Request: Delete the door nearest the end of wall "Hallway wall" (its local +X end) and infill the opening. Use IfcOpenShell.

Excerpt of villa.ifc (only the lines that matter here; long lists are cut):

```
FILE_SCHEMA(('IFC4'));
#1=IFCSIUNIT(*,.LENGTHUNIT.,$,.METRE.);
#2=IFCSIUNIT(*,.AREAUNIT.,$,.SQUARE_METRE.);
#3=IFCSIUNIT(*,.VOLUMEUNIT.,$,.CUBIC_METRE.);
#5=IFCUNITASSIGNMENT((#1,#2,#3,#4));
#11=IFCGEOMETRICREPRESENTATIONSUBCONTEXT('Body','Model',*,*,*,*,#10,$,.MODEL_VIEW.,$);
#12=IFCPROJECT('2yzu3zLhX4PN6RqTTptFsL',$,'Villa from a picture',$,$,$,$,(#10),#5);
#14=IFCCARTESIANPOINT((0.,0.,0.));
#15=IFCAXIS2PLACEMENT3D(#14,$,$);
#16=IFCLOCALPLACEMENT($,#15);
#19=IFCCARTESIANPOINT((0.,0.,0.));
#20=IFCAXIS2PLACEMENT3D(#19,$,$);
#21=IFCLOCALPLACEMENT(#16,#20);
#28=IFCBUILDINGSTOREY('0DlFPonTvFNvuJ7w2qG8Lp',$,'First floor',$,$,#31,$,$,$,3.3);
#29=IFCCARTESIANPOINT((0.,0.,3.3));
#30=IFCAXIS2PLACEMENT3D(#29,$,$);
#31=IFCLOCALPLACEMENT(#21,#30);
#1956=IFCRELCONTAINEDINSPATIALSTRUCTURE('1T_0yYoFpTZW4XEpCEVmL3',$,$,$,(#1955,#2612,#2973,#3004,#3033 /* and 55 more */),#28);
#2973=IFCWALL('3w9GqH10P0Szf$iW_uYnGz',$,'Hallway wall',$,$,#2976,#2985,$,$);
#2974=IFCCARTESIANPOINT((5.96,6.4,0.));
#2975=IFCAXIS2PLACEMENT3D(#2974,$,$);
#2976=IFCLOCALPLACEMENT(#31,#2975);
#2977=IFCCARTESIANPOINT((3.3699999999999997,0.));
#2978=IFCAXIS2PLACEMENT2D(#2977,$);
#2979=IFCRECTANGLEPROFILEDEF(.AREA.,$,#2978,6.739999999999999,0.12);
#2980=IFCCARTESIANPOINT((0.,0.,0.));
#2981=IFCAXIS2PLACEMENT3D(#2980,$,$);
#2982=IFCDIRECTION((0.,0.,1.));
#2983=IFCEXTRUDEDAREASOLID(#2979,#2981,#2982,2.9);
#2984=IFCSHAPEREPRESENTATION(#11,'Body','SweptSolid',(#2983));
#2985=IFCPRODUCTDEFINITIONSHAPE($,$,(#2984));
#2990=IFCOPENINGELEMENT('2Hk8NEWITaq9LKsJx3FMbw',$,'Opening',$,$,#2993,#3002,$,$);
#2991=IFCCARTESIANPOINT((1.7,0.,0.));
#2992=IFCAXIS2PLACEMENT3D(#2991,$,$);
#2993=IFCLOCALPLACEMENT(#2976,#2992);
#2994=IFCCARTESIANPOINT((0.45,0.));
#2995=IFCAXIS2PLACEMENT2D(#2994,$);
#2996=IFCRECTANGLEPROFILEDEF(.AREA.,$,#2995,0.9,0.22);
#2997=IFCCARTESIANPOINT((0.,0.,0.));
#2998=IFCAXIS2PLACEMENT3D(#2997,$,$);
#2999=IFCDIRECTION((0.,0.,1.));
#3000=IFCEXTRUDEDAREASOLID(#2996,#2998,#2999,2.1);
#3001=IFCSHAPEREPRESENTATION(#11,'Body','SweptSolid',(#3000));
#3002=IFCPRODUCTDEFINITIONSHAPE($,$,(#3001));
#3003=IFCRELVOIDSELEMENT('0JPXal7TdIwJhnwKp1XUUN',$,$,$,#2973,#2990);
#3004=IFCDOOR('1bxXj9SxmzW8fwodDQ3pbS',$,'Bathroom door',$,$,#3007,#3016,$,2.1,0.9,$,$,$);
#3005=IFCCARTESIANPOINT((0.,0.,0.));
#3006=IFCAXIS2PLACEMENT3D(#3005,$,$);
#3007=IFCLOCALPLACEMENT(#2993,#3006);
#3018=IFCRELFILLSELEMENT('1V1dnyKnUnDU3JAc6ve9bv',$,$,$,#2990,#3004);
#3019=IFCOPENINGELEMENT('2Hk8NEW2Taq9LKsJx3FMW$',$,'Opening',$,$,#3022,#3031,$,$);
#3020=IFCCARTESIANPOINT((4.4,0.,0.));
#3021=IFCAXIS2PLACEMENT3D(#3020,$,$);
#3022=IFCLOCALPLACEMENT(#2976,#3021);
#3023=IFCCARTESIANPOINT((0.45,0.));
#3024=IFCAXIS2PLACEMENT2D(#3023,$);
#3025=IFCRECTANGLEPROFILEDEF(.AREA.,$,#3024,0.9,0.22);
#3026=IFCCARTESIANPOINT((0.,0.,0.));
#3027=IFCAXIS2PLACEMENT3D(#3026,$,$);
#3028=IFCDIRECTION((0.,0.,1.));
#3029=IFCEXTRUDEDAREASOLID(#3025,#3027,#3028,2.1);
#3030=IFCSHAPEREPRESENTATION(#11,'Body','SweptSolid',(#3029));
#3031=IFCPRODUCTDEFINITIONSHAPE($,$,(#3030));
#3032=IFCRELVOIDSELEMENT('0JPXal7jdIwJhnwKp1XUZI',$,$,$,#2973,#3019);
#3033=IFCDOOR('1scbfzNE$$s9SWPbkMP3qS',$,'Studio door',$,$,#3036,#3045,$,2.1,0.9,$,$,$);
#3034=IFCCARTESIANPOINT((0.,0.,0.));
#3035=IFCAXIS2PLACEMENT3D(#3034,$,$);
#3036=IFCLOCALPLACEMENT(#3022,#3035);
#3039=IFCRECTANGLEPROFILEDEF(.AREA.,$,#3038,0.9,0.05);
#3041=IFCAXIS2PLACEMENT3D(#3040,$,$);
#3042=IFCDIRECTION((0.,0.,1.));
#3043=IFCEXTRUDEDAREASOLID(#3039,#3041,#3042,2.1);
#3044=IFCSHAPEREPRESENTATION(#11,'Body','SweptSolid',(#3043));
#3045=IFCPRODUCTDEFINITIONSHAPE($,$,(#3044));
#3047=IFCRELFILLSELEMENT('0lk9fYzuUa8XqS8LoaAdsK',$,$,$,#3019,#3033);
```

```python
import ifcopenshell
import ifcopenshell.api.feature
import ifcopenshell.api.root
import ifcopenshell.geom
import ifcopenshell.util.shape

model = ifcopenshell.open("villa.ifc")
settings = ifcopenshell.geom.settings()


def volume(element):
    """Net volume in cubic metres, openings subtracted."""
    shape = ifcopenshell.geom.create_shape(settings, element)
    return ifcopenshell.util.shape.get_volume(shape.geometry)


door = model.by_guid("1scbfzNE$$s9SWPbkMP3qS")
opening = door.FillsVoids[0].RelatingOpeningElement
wall = opening.VoidsElements[0].RelatingBuildingElement
before = volume(wall)

ifcopenshell.api.root.remove_product(model, product=door)
ifcopenshell.api.feature.remove_feature(model, feature=opening)

after = volume(wall)

print(f"wall volume {before:.3f} -> {after:.3f} m3")

model.write("villa_edited.ifc")
```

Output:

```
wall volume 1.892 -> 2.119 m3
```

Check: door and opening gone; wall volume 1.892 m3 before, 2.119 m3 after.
